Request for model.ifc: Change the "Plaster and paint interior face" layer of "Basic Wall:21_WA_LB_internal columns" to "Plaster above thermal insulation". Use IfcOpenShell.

First a look at what the model holds.

```python
import ifcopenshell
import ifcopenshell.util.element

model = ifcopenshell.open("model.ifc")
print(model.schema)
for layer_set in model.by_type("IfcMaterialLayerSet"):
    if layer_set.LayerSetName == "Basic Wall:21_WA_LB_internal columns":
        for layer in layer_set.MaterialLayers:
            print(layer.id(), layer.Material and layer.Material.Name, layer.LayerThickness, sep=" | ")
        print(len(ifcopenshell.util.element.get_elements_by_material(model, layer_set)), "elements and types use it")
print(sorted(m.Name for m in model.by_type("IfcMaterial") if m.Name)[:60])
```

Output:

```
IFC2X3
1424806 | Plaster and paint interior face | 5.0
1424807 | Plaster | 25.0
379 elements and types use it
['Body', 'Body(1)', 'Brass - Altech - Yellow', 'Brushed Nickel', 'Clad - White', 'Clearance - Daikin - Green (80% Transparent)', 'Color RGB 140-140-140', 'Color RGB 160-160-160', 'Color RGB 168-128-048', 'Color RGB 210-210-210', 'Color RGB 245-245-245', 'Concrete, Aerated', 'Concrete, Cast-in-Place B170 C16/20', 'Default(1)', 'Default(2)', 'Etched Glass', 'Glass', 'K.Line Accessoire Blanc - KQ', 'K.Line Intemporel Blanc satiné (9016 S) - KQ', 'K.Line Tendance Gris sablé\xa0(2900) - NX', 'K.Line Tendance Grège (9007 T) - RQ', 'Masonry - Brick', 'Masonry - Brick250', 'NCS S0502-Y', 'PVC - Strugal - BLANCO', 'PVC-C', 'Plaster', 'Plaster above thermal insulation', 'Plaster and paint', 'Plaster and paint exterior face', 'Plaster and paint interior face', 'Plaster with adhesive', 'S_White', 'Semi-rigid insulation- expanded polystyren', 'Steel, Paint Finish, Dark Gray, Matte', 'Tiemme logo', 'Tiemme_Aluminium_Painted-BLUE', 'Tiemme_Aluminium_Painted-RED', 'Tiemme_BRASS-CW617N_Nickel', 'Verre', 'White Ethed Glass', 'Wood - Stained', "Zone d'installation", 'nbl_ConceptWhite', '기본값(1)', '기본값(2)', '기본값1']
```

```python
import ifcopenshell
import ifcopenshell.api.material

model = ifcopenshell.open("model.ifc")

layer_set = next(s for s in model.by_type("IfcMaterialLayerSet") if s.LayerSetName == "Basic Wall:21_WA_LB_internal columns")
layer = next(l for l in layer_set.MaterialLayers if l.Material and l.Material.Name == "Plaster and paint interior face")
material = next(m for m in model.by_type("IfcMaterial") if m.Name == "Plaster above thermal insulation")

# Point this one layer at the other material; renaming the old one would change it everywhere.
ifcopenshell.api.material.edit_layer(model, layer=layer, attributes={}, material=material)

print([l.Material.Name if l.Material else None for l in layer_set.MaterialLayers])

model.write("model-out.ifc")
```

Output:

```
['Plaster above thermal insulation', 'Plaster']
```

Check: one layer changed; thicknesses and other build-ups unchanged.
